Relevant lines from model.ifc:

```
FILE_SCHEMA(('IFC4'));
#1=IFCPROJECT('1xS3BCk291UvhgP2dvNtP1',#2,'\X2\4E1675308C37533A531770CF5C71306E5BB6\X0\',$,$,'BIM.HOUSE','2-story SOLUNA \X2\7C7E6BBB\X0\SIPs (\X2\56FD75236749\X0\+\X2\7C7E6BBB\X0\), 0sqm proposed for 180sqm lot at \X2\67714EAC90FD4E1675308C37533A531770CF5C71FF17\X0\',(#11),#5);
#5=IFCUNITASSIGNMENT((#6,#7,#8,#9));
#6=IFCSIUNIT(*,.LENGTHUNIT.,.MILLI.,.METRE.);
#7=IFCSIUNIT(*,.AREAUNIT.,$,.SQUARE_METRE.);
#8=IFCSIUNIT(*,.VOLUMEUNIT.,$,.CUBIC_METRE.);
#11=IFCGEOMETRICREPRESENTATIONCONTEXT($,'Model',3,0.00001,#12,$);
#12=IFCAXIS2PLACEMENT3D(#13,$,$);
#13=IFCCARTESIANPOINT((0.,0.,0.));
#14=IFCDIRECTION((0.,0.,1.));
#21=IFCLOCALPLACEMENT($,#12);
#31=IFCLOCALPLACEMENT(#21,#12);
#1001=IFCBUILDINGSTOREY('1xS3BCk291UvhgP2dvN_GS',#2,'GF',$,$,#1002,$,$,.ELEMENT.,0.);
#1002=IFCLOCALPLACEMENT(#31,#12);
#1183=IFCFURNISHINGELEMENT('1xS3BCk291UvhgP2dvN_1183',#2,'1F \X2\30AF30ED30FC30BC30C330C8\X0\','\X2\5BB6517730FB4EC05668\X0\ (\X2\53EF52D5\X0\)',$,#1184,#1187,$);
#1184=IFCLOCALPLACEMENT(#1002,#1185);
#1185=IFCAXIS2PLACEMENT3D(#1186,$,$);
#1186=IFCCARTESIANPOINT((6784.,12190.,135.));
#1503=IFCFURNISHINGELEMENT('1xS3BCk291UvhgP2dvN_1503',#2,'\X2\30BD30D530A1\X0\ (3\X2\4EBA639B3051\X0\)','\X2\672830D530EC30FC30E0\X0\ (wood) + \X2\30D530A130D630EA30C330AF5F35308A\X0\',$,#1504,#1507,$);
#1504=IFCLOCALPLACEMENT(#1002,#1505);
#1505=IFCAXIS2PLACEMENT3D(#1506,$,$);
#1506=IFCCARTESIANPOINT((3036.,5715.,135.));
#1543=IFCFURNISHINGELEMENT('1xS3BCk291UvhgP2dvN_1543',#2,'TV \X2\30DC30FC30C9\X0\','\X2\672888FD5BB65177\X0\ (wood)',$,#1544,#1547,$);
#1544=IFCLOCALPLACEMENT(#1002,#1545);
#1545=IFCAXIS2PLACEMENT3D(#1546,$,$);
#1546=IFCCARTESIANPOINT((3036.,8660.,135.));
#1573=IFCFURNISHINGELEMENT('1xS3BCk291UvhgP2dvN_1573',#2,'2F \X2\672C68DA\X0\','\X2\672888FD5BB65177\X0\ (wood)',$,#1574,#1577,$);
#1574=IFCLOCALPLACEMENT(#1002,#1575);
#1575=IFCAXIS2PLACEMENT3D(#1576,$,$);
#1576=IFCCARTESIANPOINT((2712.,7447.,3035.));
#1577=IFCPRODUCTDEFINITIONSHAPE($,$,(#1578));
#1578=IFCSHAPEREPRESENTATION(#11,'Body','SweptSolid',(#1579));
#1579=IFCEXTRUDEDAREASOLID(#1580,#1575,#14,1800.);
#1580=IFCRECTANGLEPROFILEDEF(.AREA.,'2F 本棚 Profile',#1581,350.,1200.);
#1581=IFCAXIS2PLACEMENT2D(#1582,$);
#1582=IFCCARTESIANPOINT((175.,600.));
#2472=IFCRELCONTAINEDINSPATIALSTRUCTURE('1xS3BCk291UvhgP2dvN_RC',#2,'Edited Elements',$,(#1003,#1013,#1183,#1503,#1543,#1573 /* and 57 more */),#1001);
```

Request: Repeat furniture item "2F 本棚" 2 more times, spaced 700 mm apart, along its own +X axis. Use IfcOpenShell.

```python
import ifcopenshell
import ifcopenshell.api.geometry
import ifcopenshell.api.root
import ifcopenshell.util.element
import ifcopenshell.util.placement
import ifcopenshell.util.unit

model = ifcopenshell.open("model.ifc")
unit_scale = ifcopenshell.util.unit.calculate_unit_scale(model)


def reuse_history(source, copy):
    """copy_class also copies each property set's owner history, people and application; keep the originals."""
    for rel in copy.IsDefinedBy:
        if rel.is_a("IfcRelDefinesByProperties") and (history := rel.RelatingPropertyDefinition.OwnerHistory):
            rel.RelatingPropertyDefinition.OwnerHistory = source.OwnerHistory
            ifcopenshell.util.element.remove_deep2(model, history)


source = model.by_guid("1xS3BCk291UvhgP2dvN_1573")
base = ifcopenshell.util.placement.get_local_placement(source.ObjectPlacement)
step = base[:3, 0] * 0.7 / unit_scale

for i in range(1, 3):
    copy = ifcopenshell.api.root.copy_class(model, product=source)
    copy.Representation = ifcopenshell.util.element.copy_deep(
        model, source.Representation, exclude=["IfcGeometricRepresentationContext", "IfcRepresentationMap"]
    )
    reuse_history(source, copy)
    matrix = base.copy()
    matrix[:3, 3] += i * step
    print("added at", matrix[:3, 3].round(3) + 0.0)
    ifcopenshell.api.geometry.edit_object_placement(model, product=copy, matrix=matrix, is_si=False)

model.write("model_updated.ifc")
```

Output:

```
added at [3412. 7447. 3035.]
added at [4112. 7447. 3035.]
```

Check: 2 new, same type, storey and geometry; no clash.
